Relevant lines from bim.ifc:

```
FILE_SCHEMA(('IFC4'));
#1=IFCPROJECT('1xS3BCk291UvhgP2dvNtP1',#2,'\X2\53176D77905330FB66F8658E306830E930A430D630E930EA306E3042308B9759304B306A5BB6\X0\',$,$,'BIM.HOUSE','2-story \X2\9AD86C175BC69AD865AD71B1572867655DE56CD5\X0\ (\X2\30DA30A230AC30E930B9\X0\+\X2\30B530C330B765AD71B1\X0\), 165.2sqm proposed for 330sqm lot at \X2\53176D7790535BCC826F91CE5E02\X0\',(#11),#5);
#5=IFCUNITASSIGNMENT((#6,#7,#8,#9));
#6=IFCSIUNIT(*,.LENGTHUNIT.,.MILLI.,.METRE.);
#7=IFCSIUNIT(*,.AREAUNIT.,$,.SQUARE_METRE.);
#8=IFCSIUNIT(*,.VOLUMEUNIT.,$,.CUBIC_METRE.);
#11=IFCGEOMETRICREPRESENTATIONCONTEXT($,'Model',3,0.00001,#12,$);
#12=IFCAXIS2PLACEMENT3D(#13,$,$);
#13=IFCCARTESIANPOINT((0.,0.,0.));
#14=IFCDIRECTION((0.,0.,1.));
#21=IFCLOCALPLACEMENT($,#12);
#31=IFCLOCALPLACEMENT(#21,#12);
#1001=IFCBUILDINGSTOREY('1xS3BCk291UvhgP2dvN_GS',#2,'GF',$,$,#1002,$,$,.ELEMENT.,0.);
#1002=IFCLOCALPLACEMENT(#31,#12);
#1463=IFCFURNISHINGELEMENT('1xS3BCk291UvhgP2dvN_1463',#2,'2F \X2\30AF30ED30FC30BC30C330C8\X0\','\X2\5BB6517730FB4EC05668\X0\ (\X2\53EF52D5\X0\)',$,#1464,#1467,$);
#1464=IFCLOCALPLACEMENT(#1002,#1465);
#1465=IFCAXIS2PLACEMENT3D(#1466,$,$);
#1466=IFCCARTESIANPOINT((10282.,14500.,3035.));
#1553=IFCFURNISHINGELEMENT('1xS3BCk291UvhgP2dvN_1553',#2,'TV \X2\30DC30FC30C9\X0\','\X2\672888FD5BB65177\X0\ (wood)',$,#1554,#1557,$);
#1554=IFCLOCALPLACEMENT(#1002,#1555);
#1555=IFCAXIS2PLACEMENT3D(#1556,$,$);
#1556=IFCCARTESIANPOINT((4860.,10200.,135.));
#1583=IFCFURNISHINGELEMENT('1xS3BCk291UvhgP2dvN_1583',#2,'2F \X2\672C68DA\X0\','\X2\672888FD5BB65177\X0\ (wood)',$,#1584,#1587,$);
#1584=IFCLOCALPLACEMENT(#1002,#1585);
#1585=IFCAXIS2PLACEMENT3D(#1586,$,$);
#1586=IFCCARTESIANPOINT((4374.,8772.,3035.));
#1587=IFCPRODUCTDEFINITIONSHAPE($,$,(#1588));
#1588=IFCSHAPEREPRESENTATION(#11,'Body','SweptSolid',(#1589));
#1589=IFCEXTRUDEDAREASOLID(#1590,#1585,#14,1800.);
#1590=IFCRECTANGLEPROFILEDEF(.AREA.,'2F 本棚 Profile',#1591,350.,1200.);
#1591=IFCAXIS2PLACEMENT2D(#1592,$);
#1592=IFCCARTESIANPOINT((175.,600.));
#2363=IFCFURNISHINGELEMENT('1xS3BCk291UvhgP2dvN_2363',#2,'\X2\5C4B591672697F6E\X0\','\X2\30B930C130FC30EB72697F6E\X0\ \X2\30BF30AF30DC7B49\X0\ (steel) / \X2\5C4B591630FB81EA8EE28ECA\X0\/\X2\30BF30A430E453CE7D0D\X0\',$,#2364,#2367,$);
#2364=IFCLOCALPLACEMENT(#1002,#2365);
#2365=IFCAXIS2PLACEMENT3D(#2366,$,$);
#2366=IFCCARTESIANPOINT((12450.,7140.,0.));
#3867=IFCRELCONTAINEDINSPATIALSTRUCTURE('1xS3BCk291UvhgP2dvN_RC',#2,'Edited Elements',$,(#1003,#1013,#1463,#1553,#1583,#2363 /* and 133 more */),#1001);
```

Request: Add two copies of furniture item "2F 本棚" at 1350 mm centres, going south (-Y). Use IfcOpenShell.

```python
import numpy as np
import ifcopenshell
import ifcopenshell.api.geometry
import ifcopenshell.api.root
import ifcopenshell.util.element
import ifcopenshell.util.placement

model = ifcopenshell.open("bim.ifc")


def reuse_history(source, copy):
    """copy_class also copies each property set's owner history, people and application; keep the originals."""
    for rel in copy.IsDefinedBy:
        if rel.is_a("IfcRelDefinesByProperties") and (history := rel.RelatingPropertyDefinition.OwnerHistory):
            rel.RelatingPropertyDefinition.OwnerHistory = source.OwnerHistory
            ifcopenshell.util.element.remove_deep2(model, history)


source = model.by_guid("1xS3BCk291UvhgP2dvN_1583")
base = ifcopenshell.util.placement.get_local_placement(source.ObjectPlacement)
step = np.array([0.0, -1.0, 0.0]) * 1350.0

for i in range(1, 3):
    copy = ifcopenshell.api.root.copy_class(model, product=source)
    copy.Representation = ifcopenshell.util.element.copy_deep(
        model, source.Representation, exclude=["IfcGeometricRepresentationContext", "IfcRepresentationMap"]
    )
    reuse_history(source, copy)
    matrix = base.copy()
    matrix[:3, 3] += i * step
    print("added at", matrix[:3, 3].round(3) + 0.0)
    ifcopenshell.api.geometry.edit_object_placement(model, product=copy, matrix=matrix, is_si=False)

model.write("bim_rev.ifc")
```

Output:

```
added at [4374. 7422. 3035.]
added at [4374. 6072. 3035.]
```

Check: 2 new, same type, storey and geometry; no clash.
